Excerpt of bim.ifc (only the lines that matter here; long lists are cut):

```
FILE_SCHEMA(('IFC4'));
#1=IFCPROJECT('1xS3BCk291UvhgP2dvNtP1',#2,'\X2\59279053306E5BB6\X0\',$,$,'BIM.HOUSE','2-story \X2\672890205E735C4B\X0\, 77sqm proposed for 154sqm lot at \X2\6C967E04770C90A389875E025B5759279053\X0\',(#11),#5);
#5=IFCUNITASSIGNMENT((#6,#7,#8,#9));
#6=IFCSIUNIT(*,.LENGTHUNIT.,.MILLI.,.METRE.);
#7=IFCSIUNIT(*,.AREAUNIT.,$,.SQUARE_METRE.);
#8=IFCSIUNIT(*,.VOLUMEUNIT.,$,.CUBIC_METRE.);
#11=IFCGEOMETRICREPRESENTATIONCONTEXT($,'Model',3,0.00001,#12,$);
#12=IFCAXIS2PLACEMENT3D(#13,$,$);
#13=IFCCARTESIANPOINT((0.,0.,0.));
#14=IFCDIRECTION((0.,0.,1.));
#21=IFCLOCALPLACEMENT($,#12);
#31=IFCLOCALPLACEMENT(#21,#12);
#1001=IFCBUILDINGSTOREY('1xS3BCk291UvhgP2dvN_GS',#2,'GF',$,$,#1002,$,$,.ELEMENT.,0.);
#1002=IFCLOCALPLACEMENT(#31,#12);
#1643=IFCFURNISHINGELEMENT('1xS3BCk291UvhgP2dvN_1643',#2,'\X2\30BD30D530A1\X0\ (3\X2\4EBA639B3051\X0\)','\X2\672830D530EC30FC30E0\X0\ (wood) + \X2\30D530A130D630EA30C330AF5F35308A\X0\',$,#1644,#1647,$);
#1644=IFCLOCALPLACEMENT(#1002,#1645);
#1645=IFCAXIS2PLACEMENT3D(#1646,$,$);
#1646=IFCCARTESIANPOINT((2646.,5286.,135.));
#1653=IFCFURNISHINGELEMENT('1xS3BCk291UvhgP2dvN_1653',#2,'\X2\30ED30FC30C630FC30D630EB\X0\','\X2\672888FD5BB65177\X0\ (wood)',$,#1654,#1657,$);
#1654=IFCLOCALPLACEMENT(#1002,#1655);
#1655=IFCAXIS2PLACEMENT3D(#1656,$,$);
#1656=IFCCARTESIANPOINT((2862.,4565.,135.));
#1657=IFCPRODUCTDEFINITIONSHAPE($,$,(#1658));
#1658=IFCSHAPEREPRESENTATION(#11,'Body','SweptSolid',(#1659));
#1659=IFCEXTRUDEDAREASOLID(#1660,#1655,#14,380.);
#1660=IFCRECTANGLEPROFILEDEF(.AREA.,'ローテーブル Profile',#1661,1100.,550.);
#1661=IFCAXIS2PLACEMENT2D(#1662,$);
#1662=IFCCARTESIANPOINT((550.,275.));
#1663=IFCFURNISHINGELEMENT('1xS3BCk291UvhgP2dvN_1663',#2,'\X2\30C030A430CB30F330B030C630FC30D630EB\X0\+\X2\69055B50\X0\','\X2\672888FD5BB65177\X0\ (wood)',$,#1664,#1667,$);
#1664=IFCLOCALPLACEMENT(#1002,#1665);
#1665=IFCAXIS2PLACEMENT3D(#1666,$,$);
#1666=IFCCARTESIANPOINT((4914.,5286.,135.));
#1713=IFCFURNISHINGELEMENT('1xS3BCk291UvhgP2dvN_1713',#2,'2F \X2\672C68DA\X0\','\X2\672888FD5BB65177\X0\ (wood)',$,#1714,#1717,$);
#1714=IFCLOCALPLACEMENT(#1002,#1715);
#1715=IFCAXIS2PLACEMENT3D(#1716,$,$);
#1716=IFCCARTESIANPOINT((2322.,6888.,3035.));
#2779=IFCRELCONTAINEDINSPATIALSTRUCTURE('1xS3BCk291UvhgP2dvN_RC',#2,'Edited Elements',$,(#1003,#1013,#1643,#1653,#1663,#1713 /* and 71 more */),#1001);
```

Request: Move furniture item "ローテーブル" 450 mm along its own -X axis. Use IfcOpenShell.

```python
import ifcopenshell
import ifcopenshell.api.geometry
import ifcopenshell.util.placement

model = ifcopenshell.open("bim.ifc")

item = model.by_id(1653)
matrix = ifcopenshell.util.placement.get_local_placement(item.ObjectPlacement)
matrix[:3, 3] -= matrix[:3, 0] * 450.0
ifcopenshell.api.geometry.edit_object_placement(model, product=item, matrix=matrix, is_si=False)

print(ifcopenshell.util.placement.get_local_placement(item.ObjectPlacement).round(3) + 0.0)

model.write("bim-out.ifc")
```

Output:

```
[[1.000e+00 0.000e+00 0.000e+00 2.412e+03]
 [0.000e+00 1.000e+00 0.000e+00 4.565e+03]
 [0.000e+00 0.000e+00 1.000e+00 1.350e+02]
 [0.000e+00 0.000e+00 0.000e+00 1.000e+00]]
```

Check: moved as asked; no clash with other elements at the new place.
